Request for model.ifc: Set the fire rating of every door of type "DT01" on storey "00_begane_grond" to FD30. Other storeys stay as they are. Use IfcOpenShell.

First a look at what the model holds.

```python
import ifcopenshell
import ifcopenshell.util.element

model = ifcopenshell.open("model.ifc")
print(model.schema)
storey = next(s for s in model.by_type("IfcBuildingStorey") if s.Name == "00_begane_grond")
doors = [e for e in ifcopenshell.util.element.get_decomposition(storey) if e.is_a("IfcDoor")]
seen = {}
for e in doors:
    element_type = ifcopenshell.util.element.get_type(e)
    key = (element_type.Name if element_type != e and element_type else None, ifcopenshell.util.element.get_pset(e, "Pset_DoorCommon", "FireRating"))
    seen[key] = seen.get(key, 0) + 1
for (name, value), count in sorted(seen.items(), key=str):
    print(count, "x", name, "|", value)
```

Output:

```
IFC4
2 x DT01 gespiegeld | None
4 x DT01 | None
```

```python
import ifcopenshell
import ifcopenshell.api.pset
import ifcopenshell.util.element

model = ifcopenshell.open("model.ifc")

storey = next(s for s in model.by_type("IfcBuildingStorey") if s.Name == "00_begane_grond")
doors = [e for e in ifcopenshell.util.element.get_decomposition(storey) if e.is_a("IfcDoor")]

count = 0
for e in doors:
    element_type = ifcopenshell.util.element.get_type(e)
    if element_type in (None, e) or element_type.Name != "DT01":
        continue
    # add_pset returns the element's existing set when there is one.
    pset = ifcopenshell.api.pset.add_pset(model, product=e, name="Pset_DoorCommon")
    ifcopenshell.api.pset.edit_pset(model, pset=pset, properties={"FireRating": "FD30"})
    count += 1

print(count, "doors updated")

model.write("model_updated.ifc")
```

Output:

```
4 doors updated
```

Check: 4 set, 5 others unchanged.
